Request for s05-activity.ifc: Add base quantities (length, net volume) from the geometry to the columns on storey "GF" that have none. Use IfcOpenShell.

First a look at what the model holds.

```python
import ifcopenshell
import ifcopenshell.util.element
import ifcopenshell.util.unit

model = ifcopenshell.open("s05-activity.ifc")
print(model.schema)
for unit_type in ("LENGTHUNIT", "AREAUNIT", "VOLUMEUNIT"):
    print(unit_type, ifcopenshell.util.unit.calculate_unit_scale(model, unit_type))
storey = next(s for s in model.by_type("IfcBuildingStorey") if s.Name == "GF")
columns = [e for e in ifcopenshell.util.element.get_decomposition(storey) if e.is_a("IfcColumn")]
for e in sorted(columns, key=lambda e: e.id()):
    print(e.id(), e.is_a(), e.Name, list(ifcopenshell.util.element.get_psets(e, qtos_only=True)), sep=" | ")
```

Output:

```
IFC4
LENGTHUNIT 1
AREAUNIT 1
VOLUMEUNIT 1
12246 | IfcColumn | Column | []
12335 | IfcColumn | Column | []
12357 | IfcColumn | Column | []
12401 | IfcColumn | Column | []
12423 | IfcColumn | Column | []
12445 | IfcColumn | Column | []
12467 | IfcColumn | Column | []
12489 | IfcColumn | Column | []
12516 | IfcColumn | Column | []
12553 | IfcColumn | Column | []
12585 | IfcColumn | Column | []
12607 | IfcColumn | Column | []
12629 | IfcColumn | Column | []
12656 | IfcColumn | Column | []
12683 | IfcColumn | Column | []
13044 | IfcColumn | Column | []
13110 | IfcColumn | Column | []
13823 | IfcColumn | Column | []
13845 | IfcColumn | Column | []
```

```python
import ifcopenshell
import ifcopenshell.api.pset
import ifcopenshell.geom
import ifcopenshell.util.element
import ifcopenshell.util.shape
import ifcopenshell.util.unit

model = ifcopenshell.open("s05-activity.ifc")
unit_scale = ifcopenshell.util.unit.calculate_unit_scale(model)
volume_scale = ifcopenshell.util.unit.calculate_unit_scale(model, "VOLUMEUNIT")
settings = ifcopenshell.geom.settings()

storey = next(s for s in model.by_type("IfcBuildingStorey") if s.Name == "GF")
columns = [e for e in ifcopenshell.util.element.get_decomposition(storey) if e.is_a("IfcColumn")]

for e in sorted(columns, key=lambda e: e.id()):
    if ifcopenshell.util.element.get_psets(e, qtos_only=True, should_inherit=False):
        continue
    # Geometry comes back in metres, in the element's own axes.
    shape = ifcopenshell.geom.create_shape(settings, e)
    values = {
        "Length": ifcopenshell.util.shape.get_z(shape.geometry) / unit_scale,
        "NetVolume": ifcopenshell.util.shape.get_volume(shape.geometry) / volume_scale,
    }
    qto = ifcopenshell.api.pset.add_qto(model, product=e, name="Qto_ColumnBaseQuantities")
    ifcopenshell.api.pset.edit_qto(model, qto=qto, properties=values)
    print(e.id(), {k: round(v, 3) for k, v in values.items()})

model.write("s05-activity_rev.ifc")
```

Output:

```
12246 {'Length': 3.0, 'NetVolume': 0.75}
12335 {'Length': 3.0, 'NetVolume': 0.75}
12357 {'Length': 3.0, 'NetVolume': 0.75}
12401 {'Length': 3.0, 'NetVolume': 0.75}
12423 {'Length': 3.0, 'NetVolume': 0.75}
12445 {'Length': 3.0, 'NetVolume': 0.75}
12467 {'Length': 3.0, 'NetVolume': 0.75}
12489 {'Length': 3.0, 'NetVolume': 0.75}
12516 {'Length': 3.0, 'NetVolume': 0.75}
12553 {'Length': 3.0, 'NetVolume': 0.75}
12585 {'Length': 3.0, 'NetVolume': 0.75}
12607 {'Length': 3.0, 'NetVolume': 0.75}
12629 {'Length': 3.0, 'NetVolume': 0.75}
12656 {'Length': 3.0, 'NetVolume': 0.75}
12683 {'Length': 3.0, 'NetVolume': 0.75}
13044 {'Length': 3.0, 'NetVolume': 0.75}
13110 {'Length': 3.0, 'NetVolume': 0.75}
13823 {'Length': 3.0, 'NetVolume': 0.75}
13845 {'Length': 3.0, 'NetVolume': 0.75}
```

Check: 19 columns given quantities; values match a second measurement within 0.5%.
